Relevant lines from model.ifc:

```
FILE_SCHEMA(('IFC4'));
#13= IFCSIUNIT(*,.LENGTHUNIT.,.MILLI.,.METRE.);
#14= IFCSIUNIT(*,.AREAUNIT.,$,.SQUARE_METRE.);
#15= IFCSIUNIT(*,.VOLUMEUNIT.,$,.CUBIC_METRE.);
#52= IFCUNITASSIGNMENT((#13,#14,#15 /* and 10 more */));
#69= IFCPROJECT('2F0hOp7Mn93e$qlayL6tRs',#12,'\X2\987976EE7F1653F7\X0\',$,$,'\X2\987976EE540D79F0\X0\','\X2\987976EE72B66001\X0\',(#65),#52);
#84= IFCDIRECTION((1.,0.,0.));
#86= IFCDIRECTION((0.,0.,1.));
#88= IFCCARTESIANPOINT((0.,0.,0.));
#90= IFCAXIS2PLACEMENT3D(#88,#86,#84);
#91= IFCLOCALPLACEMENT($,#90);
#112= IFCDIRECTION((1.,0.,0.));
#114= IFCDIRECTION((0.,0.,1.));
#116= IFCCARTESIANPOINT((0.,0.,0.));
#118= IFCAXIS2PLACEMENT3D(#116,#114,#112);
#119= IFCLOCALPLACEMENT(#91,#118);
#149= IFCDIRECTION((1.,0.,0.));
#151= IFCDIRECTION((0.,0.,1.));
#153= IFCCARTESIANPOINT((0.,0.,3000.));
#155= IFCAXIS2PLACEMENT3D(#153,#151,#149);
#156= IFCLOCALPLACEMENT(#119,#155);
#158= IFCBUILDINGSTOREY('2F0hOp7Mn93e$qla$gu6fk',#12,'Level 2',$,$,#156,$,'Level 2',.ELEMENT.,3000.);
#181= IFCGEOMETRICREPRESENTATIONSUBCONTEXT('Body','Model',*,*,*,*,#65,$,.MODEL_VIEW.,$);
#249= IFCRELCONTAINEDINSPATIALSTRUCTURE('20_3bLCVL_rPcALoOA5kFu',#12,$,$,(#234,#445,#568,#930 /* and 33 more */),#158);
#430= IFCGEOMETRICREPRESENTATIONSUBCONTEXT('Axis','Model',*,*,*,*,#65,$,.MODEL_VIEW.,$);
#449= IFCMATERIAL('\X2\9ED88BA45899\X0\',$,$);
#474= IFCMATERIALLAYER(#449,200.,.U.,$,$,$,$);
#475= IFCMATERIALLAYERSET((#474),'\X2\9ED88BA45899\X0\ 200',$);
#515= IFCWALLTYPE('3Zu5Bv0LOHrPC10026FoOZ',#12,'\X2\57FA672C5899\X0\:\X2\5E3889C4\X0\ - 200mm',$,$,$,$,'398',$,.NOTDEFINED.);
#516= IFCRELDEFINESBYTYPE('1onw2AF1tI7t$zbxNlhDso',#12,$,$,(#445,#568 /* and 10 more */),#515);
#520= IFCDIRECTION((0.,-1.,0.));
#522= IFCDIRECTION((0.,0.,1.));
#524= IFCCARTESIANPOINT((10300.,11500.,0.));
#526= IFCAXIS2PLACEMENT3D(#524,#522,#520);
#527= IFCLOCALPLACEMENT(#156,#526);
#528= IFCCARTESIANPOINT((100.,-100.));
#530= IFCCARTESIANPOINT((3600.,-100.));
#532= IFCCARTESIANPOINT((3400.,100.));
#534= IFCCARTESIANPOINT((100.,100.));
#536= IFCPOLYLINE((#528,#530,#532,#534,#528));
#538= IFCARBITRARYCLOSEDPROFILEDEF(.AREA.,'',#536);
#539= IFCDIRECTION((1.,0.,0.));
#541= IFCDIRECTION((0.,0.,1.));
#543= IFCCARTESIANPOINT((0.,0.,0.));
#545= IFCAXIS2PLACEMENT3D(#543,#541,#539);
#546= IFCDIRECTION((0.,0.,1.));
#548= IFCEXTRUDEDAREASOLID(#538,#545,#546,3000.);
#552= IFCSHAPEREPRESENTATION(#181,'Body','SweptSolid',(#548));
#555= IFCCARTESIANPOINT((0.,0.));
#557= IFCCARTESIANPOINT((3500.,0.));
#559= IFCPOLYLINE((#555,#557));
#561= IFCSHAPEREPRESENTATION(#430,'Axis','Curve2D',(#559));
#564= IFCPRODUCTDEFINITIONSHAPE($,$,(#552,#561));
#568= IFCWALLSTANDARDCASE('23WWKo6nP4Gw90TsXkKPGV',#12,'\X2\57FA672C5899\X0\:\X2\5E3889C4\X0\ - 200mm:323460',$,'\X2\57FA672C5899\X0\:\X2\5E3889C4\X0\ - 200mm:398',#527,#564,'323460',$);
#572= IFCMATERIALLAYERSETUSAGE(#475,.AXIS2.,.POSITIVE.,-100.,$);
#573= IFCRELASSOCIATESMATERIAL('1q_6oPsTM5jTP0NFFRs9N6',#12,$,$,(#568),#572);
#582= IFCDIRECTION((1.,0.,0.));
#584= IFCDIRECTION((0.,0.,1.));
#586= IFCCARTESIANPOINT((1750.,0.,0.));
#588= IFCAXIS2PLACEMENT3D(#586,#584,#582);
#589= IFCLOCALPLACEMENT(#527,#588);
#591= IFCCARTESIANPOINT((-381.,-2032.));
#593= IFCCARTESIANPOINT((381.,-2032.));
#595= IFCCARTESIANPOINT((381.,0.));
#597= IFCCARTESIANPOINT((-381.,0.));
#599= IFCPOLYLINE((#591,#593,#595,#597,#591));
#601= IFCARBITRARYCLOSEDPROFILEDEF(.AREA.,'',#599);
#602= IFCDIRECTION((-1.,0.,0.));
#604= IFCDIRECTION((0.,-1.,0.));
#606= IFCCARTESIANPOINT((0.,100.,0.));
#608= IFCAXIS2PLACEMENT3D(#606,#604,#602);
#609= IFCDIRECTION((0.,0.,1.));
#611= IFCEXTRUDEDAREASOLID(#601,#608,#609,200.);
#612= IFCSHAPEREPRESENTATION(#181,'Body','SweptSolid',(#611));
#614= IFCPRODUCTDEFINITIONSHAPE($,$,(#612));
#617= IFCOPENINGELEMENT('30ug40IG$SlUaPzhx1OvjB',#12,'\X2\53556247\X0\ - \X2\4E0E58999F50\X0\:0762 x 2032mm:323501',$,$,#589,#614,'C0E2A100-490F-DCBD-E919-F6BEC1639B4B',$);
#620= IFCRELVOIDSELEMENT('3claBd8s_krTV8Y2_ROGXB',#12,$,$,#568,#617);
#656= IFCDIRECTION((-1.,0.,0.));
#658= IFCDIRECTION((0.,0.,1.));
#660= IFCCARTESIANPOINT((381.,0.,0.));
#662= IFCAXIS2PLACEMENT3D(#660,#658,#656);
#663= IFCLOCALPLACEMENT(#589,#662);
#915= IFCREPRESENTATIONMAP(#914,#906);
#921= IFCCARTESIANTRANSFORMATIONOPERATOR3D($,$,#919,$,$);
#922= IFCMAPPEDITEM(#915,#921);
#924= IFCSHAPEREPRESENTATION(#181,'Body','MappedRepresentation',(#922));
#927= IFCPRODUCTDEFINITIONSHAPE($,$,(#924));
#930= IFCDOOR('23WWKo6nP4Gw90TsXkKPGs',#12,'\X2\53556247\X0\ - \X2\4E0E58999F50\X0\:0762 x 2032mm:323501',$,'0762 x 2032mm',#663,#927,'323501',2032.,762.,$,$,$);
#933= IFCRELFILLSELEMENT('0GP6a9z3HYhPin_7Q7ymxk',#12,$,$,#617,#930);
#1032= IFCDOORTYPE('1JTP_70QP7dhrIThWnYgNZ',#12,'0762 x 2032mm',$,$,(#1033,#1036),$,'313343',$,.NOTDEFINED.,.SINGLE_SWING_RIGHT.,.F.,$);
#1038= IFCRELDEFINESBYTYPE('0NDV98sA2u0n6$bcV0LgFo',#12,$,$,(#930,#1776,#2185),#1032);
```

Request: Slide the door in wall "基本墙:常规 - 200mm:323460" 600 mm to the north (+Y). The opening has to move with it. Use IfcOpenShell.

```python
import ifcopenshell
import ifcopenshell.api.geometry
import ifcopenshell.util.placement
import ifcopenshell.util.unit

model = ifcopenshell.open("model.ifc")
unit_scale = ifcopenshell.util.unit.calculate_unit_scale(model)

door = model.by_guid("23WWKo6nP4Gw90TsXkKPGs")
opening = door.FillsVoids[0].RelatingOpeningElement
wall = opening.VoidsElements[0].RelatingBuildingElement

wall_matrix = ifcopenshell.util.placement.get_local_placement(wall.ObjectPlacement)
shift = wall_matrix[:3, 0] * -0.6 / unit_scale
before = ifcopenshell.util.placement.get_local_placement(door.ObjectPlacement)[:3, 3].copy()

# The door is placed relative to its opening, so it follows when the opening moves.
matrix = ifcopenshell.util.placement.get_local_placement(opening.ObjectPlacement)
matrix[:3, 3] += shift
ifcopenshell.api.geometry.edit_object_placement(
    model, product=opening, matrix=matrix, is_si=False, should_transform_children=True
)

after = ifcopenshell.util.placement.get_local_placement(door.ObjectPlacement)[:3, 3]
print("door moved by", (after - before).round(3) + 0.0)

model.write("model_updated.ifc")
```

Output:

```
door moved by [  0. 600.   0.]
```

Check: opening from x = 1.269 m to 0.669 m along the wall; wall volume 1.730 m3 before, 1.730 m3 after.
